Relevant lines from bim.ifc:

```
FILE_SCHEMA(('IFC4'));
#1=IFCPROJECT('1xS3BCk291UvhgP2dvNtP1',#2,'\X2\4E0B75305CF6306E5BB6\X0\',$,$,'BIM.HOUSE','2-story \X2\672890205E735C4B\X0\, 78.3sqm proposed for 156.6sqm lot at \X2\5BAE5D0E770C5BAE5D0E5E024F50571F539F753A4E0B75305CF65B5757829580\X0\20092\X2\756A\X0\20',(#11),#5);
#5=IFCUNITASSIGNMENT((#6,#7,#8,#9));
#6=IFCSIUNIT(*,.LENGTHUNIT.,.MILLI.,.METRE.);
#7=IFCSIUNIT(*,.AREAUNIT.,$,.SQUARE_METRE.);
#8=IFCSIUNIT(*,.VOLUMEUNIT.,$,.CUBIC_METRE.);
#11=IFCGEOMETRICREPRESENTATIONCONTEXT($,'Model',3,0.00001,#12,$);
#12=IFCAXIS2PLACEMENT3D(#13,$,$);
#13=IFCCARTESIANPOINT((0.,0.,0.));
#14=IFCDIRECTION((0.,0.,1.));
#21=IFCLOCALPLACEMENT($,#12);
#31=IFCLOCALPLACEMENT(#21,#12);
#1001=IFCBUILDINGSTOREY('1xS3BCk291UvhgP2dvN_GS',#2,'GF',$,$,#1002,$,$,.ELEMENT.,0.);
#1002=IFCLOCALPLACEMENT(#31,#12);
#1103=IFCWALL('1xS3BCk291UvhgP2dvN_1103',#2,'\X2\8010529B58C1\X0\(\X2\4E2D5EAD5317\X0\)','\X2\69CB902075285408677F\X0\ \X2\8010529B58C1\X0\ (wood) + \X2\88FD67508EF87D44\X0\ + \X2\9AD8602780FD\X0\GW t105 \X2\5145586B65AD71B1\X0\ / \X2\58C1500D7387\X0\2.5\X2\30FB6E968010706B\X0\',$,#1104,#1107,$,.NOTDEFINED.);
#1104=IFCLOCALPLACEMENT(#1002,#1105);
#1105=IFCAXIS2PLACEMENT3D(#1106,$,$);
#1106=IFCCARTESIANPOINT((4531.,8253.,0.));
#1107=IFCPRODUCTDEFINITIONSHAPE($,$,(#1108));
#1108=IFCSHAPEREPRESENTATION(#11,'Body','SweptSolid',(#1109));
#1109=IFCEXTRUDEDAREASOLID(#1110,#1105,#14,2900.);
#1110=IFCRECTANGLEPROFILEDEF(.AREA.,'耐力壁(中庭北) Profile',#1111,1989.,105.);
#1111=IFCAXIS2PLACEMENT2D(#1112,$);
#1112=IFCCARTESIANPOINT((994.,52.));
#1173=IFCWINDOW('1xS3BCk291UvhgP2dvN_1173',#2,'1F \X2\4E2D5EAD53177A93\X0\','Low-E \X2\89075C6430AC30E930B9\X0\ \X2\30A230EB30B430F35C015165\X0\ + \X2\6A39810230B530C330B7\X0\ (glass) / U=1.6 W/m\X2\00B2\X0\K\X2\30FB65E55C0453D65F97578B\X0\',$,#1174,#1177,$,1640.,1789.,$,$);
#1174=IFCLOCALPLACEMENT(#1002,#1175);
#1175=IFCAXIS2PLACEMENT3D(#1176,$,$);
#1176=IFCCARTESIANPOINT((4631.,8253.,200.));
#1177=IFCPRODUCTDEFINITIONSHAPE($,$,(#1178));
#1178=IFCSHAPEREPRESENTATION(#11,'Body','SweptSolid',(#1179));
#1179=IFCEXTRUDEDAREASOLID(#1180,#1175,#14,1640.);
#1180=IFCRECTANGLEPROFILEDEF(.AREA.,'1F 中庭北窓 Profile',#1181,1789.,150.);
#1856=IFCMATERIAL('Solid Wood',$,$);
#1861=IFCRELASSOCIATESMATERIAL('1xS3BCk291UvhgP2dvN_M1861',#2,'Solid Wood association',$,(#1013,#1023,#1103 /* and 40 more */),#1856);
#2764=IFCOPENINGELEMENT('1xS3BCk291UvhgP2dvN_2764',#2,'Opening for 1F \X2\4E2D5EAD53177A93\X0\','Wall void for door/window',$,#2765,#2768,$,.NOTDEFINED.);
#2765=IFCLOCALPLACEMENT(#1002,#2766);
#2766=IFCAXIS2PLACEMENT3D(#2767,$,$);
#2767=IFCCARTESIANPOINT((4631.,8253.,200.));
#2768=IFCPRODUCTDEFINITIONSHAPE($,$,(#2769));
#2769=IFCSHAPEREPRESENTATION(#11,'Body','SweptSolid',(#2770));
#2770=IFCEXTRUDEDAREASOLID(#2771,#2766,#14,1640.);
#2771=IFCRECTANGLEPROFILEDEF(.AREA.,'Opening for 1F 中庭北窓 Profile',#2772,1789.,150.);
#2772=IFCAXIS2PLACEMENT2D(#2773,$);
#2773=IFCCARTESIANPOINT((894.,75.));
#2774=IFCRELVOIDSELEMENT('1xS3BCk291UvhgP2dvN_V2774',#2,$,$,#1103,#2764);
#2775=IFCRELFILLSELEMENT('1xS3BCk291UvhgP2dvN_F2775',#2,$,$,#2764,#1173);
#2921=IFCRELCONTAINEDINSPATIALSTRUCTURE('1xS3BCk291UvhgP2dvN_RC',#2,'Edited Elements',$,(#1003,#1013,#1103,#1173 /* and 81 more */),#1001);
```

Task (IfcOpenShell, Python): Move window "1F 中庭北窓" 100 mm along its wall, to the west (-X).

```python
import ifcopenshell
import ifcopenshell.api.geometry
import ifcopenshell.util.placement
import ifcopenshell.util.unit

model = ifcopenshell.open("bim.ifc")
unit_scale = ifcopenshell.util.unit.calculate_unit_scale(model)

window = model.by_id(1173)
opening = window.FillsVoids[0].RelatingOpeningElement
wall = opening.VoidsElements[0].RelatingBuildingElement

wall_matrix = ifcopenshell.util.placement.get_local_placement(wall.ObjectPlacement)
shift = wall_matrix[:3, 0] * -0.1 / unit_scale
before = ifcopenshell.util.placement.get_local_placement(window.ObjectPlacement)[:3, 3].copy()

# The window is not placed relative to its opening, so move both.
for product in (opening, window):
    matrix = ifcopenshell.util.placement.get_local_placement(product.ObjectPlacement)
    matrix[:3, 3] += shift
    ifcopenshell.api.geometry.edit_object_placement(model, product=product, matrix=matrix, is_si=False)

after = ifcopenshell.util.placement.get_local_placement(window.ObjectPlacement)[:3, 3]
print("window moved by", (after - before).round(3) + 0.0)

model.write("bim_rev.ifc")
```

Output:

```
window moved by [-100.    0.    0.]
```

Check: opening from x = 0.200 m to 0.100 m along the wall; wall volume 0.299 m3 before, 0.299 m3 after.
